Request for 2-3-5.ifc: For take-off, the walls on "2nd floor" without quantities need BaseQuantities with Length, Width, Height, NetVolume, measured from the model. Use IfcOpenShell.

First a look at what the model holds.

```python
import ifcopenshell
import ifcopenshell.util.element
import ifcopenshell.util.unit

model = ifcopenshell.open("2-3-5.ifc")
print(model.schema)
for unit_type in ("LENGTHUNIT", "AREAUNIT", "VOLUMEUNIT"):
    print(unit_type, ifcopenshell.util.unit.calculate_unit_scale(model, unit_type))
storey = next(s for s in model.by_type("IfcBuildingStorey") if s.Name == "2nd floor")
walls = [e for e in ifcopenshell.util.element.get_decomposition(storey) if e.is_a("IfcWall")]
for e in sorted(walls, key=lambda e: e.id()):
    print(e.id(), e.is_a(), e.Name, list(ifcopenshell.util.element.get_psets(e, qtos_only=True)), sep=" | ")
```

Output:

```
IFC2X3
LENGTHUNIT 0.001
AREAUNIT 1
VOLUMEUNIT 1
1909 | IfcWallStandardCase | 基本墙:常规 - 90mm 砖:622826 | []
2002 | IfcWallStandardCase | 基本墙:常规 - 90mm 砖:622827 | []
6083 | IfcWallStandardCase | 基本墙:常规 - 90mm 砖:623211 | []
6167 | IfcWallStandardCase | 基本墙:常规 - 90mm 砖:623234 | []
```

```python
import ifcopenshell
import ifcopenshell.api.pset
import ifcopenshell.geom
import ifcopenshell.util.element
import ifcopenshell.util.shape
import ifcopenshell.util.unit

model = ifcopenshell.open("2-3-5.ifc")
unit_scale = ifcopenshell.util.unit.calculate_unit_scale(model)
volume_scale = ifcopenshell.util.unit.calculate_unit_scale(model, "VOLUMEUNIT")
settings = ifcopenshell.geom.settings()

storey = next(s for s in model.by_type("IfcBuildingStorey") if s.Name == "2nd floor")
walls = [e for e in ifcopenshell.util.element.get_decomposition(storey) if e.is_a("IfcWall")]

for e in sorted(walls, key=lambda e: e.id()):
    if ifcopenshell.util.element.get_psets(e, qtos_only=True, should_inherit=False):
        continue
    # Geometry comes back in metres, in the element's own axes.
    shape = ifcopenshell.geom.create_shape(settings, e)
    values = {
        "Length": ifcopenshell.util.shape.get_x(shape.geometry) / unit_scale,
        "Width": ifcopenshell.util.shape.get_y(shape.geometry) / unit_scale,
        "Height": ifcopenshell.util.shape.get_z(shape.geometry) / unit_scale,
        "NetVolume": ifcopenshell.util.shape.get_volume(shape.geometry) / volume_scale,
    }
    qto = ifcopenshell.api.pset.add_qto(model, product=e, name="BaseQuantities")
    ifcopenshell.api.pset.edit_qto(model, qto=qto, properties=values)
    print(e.id(), {k: round(v, 3) for k, v in values.items()})

model.write("2-3-5_updated.ifc")
```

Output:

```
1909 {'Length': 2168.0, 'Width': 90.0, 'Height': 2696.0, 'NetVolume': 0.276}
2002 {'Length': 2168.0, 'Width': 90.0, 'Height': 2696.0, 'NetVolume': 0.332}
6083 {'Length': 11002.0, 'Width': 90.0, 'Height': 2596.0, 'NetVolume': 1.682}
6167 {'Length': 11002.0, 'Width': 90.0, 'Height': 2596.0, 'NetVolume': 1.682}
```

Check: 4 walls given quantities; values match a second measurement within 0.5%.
